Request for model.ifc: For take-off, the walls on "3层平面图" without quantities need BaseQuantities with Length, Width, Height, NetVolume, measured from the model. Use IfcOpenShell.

First a look at what the model holds.

```python
import ifcopenshell
import ifcopenshell.util.element
import ifcopenshell.util.unit

model = ifcopenshell.open("model.ifc")
print(model.schema)
for unit_type in ("LENGTHUNIT", "AREAUNIT", "VOLUMEUNIT"):
    print(unit_type, ifcopenshell.util.unit.calculate_unit_scale(model, unit_type))
storey = next(s for s in model.by_type("IfcBuildingStorey") if s.Name == "3层平面图")
walls = [e for e in ifcopenshell.util.element.get_decomposition(storey) if e.is_a("IfcWall")]
for e in sorted(walls, key=lambda e: e.id()):
    print(e.id(), e.is_a(), e.Name, list(ifcopenshell.util.element.get_psets(e, qtos_only=True)), sep=" | ")
```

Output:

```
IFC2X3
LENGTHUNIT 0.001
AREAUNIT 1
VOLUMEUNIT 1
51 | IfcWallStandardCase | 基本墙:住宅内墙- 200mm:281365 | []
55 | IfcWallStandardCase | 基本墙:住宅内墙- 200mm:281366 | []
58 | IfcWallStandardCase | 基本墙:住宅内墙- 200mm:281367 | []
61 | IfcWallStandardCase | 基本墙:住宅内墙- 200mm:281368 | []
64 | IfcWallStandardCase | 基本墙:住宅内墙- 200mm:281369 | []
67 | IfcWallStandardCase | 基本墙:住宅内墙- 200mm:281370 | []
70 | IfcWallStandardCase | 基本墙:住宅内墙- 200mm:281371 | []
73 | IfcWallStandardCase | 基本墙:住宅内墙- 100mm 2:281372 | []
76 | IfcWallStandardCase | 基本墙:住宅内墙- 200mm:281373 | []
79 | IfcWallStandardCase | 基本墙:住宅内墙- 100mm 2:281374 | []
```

```python
import ifcopenshell
import ifcopenshell.api.pset
import ifcopenshell.geom
import ifcopenshell.util.element
import ifcopenshell.util.shape
import ifcopenshell.util.unit

model = ifcopenshell.open("model.ifc")
unit_scale = ifcopenshell.util.unit.calculate_unit_scale(model)
volume_scale = ifcopenshell.util.unit.calculate_unit_scale(model, "VOLUMEUNIT")
settings = ifcopenshell.geom.settings()

storey = next(s for s in model.by_type("IfcBuildingStorey") if s.Name == "3层平面图")
walls = [e for e in ifcopenshell.util.element.get_decomposition(storey) if e.is_a("IfcWall")]

for e in sorted(walls, key=lambda e: e.id()):
    if ifcopenshell.util.element.get_psets(e, qtos_only=True, should_inherit=False):
        continue
    # Geometry comes back in metres, in the element's own axes.
    shape = ifcopenshell.geom.create_shape(settings, e)
    values = {
        "Length": ifcopenshell.util.shape.get_x(shape.geometry) / unit_scale,
        "Width": ifcopenshell.util.shape.get_y(shape.geometry) / unit_scale,
        "Height": ifcopenshell.util.shape.get_z(shape.geometry) / unit_scale,
        "NetVolume": ifcopenshell.util.shape.get_volume(shape.geometry) / volume_scale,
    }
    qto = ifcopenshell.api.pset.add_qto(model, product=e, name="BaseQuantities")
    ifcopenshell.api.pset.edit_qto(model, qto=qto, properties=values)
    print(e.id(), {k: round(v, 3) for k, v in values.items()})

model.write("model_edited.ifc")
```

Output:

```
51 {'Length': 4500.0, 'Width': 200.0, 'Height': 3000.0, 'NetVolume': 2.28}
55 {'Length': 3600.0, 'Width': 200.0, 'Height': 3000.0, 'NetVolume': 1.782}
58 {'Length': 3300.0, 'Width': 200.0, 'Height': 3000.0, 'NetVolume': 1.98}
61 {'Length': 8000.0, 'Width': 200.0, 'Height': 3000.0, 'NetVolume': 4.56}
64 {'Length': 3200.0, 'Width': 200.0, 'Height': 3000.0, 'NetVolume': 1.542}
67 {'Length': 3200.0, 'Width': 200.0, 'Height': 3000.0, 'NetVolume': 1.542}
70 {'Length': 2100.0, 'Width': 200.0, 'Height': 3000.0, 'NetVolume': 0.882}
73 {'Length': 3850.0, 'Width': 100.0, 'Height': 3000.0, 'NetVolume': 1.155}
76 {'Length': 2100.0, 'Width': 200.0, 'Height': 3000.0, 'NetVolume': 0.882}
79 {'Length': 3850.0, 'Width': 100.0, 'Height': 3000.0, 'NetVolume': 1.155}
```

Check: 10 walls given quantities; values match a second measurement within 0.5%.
